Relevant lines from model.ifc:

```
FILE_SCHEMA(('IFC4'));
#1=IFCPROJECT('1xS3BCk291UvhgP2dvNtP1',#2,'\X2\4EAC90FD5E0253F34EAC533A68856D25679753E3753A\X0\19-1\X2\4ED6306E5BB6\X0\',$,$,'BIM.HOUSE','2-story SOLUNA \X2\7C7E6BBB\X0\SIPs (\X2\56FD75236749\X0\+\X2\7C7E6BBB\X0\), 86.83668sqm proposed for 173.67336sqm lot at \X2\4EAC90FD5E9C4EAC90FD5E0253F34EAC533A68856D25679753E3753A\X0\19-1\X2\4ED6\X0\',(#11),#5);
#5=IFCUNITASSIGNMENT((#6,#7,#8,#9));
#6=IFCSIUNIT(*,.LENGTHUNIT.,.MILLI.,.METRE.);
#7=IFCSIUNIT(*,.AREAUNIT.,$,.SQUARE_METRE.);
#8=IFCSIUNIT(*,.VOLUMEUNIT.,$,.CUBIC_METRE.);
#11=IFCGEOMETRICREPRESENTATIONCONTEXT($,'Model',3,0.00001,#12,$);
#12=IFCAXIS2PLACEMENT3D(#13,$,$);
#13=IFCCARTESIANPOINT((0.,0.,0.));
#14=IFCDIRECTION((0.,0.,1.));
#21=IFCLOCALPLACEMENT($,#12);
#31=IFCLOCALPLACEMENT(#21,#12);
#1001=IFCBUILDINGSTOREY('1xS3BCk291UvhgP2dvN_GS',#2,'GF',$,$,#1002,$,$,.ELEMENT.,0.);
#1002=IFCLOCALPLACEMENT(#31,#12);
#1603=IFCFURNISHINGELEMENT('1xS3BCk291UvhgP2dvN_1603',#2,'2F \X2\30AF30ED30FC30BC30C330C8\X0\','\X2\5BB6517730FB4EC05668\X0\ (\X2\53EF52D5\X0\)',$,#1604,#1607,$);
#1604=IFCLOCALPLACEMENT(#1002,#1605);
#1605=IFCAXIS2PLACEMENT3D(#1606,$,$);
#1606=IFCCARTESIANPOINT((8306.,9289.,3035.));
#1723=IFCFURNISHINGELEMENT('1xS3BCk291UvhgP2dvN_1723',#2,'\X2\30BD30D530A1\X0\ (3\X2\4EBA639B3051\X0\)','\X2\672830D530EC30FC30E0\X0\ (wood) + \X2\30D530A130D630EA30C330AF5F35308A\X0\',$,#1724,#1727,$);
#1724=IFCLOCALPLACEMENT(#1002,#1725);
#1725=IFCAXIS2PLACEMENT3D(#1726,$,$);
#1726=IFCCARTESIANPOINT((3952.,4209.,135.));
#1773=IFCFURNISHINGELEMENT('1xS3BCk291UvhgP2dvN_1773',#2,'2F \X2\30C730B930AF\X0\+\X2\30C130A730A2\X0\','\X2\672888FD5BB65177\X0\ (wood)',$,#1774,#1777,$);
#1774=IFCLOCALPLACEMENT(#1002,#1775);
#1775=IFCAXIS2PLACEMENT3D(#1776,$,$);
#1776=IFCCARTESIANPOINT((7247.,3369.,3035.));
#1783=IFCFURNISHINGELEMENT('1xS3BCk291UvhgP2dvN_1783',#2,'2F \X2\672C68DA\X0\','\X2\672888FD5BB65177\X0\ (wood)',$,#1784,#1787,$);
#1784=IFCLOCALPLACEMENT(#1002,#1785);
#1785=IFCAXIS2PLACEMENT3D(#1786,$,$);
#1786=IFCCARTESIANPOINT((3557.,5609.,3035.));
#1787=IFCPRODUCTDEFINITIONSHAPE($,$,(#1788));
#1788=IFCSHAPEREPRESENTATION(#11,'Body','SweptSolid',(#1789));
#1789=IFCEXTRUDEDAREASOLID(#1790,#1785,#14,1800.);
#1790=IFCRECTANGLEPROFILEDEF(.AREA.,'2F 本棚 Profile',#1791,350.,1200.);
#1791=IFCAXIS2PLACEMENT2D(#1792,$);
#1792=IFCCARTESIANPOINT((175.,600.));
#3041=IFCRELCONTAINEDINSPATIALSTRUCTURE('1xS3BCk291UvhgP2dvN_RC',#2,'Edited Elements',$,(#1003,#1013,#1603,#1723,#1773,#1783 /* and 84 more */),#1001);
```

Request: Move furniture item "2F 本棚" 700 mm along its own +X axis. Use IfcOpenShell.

```python
import ifcopenshell
import ifcopenshell.api.geometry
import ifcopenshell.util.placement
import ifcopenshell.util.unit

model = ifcopenshell.open("model.ifc")
unit_scale = ifcopenshell.util.unit.calculate_unit_scale(model)

item = model.by_guid("1xS3BCk291UvhgP2dvN_1783")
matrix = ifcopenshell.util.placement.get_local_placement(item.ObjectPlacement)
matrix[:3, 3] += matrix[:3, 0] * 0.7 / unit_scale
ifcopenshell.api.geometry.edit_object_placement(model, product=item, matrix=matrix, is_si=False)

print(ifcopenshell.util.placement.get_local_placement(item.ObjectPlacement).round(3) + 0.0)

model.write("model_rev.ifc")
```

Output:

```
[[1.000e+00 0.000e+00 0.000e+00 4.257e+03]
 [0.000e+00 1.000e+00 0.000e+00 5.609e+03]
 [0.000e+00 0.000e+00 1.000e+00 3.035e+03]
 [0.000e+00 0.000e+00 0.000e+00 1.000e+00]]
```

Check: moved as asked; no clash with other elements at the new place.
